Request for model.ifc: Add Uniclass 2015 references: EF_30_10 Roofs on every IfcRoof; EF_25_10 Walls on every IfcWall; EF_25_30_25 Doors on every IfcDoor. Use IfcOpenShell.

First a look at what the model holds.

```python
import ifcopenshell

model = ifcopenshell.open("model.ifc")
print(model.schema)
print("classifications:", [c.Name for c in model.by_type("IfcClassification")])
for ifc_class in ("IfcDoor", "IfcRoof", "IfcStair", "IfcWall", "IfcWindow"):
    print(ifc_class, len(model.by_type(ifc_class)))
```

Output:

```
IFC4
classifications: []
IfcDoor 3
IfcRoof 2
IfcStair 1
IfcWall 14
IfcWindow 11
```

```python
import ifcopenshell
import ifcopenshell.api.classification

model = ifcopenshell.open("model.ifc")

system = ifcopenshell.api.classification.add_classification(model, classification="Uniclass 2015")

codes = {
    "IfcRoof": ("EF_30_10", "Roofs"),
    "IfcWall": ("EF_25_10", "Walls"),
    "IfcDoor": ("EF_25_30_25", "Doors"),
}
for ifc_class, (code, name) in codes.items():
    products = model.by_type(ifc_class)
    ifcopenshell.api.classification.add_reference(
        model, products=products, classification=system, identification=code, name=name
    )
    print(code, len(products))

model.write("model_rev.ifc")
```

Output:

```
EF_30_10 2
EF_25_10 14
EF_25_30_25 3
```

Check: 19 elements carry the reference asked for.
